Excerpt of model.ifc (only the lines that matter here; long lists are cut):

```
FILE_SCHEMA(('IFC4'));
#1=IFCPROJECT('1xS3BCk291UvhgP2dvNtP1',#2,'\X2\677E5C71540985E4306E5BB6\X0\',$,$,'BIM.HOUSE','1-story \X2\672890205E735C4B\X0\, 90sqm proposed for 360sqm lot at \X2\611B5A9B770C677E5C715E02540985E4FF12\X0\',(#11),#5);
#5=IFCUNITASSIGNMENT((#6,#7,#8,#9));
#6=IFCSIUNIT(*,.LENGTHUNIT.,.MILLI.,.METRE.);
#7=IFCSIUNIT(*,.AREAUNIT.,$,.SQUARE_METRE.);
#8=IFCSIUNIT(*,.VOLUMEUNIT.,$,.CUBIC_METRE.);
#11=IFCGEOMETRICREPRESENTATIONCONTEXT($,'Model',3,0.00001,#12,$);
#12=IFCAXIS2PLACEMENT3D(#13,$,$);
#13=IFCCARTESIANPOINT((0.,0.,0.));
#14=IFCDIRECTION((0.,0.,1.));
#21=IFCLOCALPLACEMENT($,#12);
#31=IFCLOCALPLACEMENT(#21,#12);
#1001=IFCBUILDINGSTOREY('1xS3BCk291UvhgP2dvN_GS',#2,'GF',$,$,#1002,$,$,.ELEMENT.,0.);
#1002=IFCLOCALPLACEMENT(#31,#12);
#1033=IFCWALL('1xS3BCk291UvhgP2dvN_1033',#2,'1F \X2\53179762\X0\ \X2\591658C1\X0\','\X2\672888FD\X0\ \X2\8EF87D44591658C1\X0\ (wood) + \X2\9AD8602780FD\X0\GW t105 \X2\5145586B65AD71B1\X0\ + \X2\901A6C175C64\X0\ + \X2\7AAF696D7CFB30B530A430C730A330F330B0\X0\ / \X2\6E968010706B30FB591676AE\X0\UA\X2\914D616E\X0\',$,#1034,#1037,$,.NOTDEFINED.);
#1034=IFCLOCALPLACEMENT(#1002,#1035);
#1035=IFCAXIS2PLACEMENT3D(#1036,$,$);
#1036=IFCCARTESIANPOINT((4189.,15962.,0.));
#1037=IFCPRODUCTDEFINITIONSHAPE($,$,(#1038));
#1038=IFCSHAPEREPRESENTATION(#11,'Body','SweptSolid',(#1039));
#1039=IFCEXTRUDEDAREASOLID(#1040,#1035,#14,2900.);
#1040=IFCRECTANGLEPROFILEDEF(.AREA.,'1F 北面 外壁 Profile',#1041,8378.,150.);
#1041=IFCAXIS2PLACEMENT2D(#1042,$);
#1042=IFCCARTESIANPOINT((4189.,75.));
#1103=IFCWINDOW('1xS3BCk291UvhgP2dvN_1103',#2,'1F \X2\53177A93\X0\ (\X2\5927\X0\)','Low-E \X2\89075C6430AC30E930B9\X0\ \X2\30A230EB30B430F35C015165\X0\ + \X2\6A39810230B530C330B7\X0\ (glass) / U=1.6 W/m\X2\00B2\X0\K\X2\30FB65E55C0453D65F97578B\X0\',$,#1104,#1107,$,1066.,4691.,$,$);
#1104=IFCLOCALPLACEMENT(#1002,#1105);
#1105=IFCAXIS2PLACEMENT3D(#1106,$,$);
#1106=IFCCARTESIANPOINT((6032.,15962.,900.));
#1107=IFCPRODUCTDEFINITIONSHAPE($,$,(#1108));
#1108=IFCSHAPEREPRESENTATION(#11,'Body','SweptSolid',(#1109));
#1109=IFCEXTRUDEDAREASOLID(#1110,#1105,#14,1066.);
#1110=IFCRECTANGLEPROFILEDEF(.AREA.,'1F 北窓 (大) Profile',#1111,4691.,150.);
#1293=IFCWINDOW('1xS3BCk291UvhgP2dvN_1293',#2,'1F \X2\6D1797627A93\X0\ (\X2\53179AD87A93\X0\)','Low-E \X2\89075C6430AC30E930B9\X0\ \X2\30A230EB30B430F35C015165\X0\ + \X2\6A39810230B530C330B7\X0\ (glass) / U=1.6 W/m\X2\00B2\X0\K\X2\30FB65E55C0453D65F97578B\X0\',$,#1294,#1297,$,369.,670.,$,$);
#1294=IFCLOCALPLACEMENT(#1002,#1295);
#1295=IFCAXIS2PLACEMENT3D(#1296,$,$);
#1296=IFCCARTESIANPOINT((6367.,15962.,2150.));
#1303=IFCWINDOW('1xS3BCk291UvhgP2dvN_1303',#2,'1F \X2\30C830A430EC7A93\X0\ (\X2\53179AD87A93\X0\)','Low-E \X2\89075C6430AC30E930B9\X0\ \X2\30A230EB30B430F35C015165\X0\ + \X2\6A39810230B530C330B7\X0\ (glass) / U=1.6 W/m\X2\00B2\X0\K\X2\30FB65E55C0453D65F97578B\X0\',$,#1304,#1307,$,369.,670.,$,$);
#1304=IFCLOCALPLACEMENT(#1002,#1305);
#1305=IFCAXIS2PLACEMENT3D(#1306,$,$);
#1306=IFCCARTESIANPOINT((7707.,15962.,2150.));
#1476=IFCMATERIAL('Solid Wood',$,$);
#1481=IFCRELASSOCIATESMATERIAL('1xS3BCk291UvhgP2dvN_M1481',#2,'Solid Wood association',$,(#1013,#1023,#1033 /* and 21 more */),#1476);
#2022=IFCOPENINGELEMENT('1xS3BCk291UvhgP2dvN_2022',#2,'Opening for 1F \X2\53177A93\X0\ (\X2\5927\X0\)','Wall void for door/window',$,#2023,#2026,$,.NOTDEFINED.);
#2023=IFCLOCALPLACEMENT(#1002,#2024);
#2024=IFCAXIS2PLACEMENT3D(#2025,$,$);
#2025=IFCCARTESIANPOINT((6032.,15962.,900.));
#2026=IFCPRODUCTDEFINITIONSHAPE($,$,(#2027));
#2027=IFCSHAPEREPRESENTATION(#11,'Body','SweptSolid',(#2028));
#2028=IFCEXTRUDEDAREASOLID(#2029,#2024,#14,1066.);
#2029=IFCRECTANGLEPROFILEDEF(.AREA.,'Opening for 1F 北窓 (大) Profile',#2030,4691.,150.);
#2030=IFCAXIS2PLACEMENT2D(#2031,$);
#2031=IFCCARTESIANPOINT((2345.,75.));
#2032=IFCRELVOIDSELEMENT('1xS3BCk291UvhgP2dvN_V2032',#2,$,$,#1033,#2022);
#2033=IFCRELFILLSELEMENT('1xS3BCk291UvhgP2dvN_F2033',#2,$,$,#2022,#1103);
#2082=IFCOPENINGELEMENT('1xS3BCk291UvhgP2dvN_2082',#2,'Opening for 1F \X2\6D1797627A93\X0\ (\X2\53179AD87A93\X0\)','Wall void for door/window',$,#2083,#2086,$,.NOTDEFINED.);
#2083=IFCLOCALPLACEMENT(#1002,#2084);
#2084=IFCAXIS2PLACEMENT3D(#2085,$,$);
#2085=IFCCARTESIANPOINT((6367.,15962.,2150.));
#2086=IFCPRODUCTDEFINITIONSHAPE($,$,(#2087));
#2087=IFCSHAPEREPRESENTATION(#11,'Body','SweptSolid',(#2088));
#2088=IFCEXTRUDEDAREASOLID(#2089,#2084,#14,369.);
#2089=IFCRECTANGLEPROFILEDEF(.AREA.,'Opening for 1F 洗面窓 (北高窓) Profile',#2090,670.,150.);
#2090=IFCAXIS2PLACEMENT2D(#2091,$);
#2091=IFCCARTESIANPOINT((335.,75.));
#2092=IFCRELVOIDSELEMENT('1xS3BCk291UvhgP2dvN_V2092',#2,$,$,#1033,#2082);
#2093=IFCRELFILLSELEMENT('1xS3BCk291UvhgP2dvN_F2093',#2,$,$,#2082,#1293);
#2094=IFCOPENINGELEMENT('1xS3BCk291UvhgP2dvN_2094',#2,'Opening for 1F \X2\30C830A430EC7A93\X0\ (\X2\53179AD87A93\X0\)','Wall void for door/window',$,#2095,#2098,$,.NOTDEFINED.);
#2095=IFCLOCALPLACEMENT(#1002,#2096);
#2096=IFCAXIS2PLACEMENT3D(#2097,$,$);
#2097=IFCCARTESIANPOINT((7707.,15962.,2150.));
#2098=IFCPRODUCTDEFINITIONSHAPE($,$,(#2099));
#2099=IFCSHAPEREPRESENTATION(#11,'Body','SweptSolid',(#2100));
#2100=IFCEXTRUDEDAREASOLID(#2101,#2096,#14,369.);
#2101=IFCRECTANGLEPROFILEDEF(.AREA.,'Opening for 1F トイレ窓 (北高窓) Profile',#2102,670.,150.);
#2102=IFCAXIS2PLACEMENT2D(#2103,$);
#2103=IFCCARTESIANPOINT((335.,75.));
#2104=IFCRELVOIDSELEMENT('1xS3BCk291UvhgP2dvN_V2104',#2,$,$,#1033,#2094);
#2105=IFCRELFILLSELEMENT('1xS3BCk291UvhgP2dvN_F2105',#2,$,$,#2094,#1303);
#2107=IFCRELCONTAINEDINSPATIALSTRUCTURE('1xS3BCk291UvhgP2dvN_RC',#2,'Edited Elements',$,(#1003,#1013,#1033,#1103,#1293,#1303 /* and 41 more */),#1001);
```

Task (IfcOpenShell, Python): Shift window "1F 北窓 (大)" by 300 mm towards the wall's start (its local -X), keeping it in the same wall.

```python
import ifcopenshell
import ifcopenshell.api.geometry
import ifcopenshell.util.placement
import ifcopenshell.util.unit

model = ifcopenshell.open("model.ifc")
unit_scale = ifcopenshell.util.unit.calculate_unit_scale(model)

window = model.by_guid("1xS3BCk291UvhgP2dvN_1103")
opening = window.FillsVoids[0].RelatingOpeningElement
wall = opening.VoidsElements[0].RelatingBuildingElement

wall_matrix = ifcopenshell.util.placement.get_local_placement(wall.ObjectPlacement)
shift = wall_matrix[:3, 0] * -0.3 / unit_scale
before = ifcopenshell.util.placement.get_local_placement(window.ObjectPlacement)[:3, 3].copy()

# The window is not placed relative to its opening, so move both.
for product in (opening, window):
    matrix = ifcopenshell.util.placement.get_local_placement(product.ObjectPlacement)
    matrix[:3, 3] += shift
    ifcopenshell.api.geometry.edit_object_placement(model, product=product, matrix=matrix, is_si=False)

after = ifcopenshell.util.placement.get_local_placement(window.ObjectPlacement)[:3, 3]
print("window moved by", (after - before).round(3) + 0.0)

model.write("model_v2.ifc")
```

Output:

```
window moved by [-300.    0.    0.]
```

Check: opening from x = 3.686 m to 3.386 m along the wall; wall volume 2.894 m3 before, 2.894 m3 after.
